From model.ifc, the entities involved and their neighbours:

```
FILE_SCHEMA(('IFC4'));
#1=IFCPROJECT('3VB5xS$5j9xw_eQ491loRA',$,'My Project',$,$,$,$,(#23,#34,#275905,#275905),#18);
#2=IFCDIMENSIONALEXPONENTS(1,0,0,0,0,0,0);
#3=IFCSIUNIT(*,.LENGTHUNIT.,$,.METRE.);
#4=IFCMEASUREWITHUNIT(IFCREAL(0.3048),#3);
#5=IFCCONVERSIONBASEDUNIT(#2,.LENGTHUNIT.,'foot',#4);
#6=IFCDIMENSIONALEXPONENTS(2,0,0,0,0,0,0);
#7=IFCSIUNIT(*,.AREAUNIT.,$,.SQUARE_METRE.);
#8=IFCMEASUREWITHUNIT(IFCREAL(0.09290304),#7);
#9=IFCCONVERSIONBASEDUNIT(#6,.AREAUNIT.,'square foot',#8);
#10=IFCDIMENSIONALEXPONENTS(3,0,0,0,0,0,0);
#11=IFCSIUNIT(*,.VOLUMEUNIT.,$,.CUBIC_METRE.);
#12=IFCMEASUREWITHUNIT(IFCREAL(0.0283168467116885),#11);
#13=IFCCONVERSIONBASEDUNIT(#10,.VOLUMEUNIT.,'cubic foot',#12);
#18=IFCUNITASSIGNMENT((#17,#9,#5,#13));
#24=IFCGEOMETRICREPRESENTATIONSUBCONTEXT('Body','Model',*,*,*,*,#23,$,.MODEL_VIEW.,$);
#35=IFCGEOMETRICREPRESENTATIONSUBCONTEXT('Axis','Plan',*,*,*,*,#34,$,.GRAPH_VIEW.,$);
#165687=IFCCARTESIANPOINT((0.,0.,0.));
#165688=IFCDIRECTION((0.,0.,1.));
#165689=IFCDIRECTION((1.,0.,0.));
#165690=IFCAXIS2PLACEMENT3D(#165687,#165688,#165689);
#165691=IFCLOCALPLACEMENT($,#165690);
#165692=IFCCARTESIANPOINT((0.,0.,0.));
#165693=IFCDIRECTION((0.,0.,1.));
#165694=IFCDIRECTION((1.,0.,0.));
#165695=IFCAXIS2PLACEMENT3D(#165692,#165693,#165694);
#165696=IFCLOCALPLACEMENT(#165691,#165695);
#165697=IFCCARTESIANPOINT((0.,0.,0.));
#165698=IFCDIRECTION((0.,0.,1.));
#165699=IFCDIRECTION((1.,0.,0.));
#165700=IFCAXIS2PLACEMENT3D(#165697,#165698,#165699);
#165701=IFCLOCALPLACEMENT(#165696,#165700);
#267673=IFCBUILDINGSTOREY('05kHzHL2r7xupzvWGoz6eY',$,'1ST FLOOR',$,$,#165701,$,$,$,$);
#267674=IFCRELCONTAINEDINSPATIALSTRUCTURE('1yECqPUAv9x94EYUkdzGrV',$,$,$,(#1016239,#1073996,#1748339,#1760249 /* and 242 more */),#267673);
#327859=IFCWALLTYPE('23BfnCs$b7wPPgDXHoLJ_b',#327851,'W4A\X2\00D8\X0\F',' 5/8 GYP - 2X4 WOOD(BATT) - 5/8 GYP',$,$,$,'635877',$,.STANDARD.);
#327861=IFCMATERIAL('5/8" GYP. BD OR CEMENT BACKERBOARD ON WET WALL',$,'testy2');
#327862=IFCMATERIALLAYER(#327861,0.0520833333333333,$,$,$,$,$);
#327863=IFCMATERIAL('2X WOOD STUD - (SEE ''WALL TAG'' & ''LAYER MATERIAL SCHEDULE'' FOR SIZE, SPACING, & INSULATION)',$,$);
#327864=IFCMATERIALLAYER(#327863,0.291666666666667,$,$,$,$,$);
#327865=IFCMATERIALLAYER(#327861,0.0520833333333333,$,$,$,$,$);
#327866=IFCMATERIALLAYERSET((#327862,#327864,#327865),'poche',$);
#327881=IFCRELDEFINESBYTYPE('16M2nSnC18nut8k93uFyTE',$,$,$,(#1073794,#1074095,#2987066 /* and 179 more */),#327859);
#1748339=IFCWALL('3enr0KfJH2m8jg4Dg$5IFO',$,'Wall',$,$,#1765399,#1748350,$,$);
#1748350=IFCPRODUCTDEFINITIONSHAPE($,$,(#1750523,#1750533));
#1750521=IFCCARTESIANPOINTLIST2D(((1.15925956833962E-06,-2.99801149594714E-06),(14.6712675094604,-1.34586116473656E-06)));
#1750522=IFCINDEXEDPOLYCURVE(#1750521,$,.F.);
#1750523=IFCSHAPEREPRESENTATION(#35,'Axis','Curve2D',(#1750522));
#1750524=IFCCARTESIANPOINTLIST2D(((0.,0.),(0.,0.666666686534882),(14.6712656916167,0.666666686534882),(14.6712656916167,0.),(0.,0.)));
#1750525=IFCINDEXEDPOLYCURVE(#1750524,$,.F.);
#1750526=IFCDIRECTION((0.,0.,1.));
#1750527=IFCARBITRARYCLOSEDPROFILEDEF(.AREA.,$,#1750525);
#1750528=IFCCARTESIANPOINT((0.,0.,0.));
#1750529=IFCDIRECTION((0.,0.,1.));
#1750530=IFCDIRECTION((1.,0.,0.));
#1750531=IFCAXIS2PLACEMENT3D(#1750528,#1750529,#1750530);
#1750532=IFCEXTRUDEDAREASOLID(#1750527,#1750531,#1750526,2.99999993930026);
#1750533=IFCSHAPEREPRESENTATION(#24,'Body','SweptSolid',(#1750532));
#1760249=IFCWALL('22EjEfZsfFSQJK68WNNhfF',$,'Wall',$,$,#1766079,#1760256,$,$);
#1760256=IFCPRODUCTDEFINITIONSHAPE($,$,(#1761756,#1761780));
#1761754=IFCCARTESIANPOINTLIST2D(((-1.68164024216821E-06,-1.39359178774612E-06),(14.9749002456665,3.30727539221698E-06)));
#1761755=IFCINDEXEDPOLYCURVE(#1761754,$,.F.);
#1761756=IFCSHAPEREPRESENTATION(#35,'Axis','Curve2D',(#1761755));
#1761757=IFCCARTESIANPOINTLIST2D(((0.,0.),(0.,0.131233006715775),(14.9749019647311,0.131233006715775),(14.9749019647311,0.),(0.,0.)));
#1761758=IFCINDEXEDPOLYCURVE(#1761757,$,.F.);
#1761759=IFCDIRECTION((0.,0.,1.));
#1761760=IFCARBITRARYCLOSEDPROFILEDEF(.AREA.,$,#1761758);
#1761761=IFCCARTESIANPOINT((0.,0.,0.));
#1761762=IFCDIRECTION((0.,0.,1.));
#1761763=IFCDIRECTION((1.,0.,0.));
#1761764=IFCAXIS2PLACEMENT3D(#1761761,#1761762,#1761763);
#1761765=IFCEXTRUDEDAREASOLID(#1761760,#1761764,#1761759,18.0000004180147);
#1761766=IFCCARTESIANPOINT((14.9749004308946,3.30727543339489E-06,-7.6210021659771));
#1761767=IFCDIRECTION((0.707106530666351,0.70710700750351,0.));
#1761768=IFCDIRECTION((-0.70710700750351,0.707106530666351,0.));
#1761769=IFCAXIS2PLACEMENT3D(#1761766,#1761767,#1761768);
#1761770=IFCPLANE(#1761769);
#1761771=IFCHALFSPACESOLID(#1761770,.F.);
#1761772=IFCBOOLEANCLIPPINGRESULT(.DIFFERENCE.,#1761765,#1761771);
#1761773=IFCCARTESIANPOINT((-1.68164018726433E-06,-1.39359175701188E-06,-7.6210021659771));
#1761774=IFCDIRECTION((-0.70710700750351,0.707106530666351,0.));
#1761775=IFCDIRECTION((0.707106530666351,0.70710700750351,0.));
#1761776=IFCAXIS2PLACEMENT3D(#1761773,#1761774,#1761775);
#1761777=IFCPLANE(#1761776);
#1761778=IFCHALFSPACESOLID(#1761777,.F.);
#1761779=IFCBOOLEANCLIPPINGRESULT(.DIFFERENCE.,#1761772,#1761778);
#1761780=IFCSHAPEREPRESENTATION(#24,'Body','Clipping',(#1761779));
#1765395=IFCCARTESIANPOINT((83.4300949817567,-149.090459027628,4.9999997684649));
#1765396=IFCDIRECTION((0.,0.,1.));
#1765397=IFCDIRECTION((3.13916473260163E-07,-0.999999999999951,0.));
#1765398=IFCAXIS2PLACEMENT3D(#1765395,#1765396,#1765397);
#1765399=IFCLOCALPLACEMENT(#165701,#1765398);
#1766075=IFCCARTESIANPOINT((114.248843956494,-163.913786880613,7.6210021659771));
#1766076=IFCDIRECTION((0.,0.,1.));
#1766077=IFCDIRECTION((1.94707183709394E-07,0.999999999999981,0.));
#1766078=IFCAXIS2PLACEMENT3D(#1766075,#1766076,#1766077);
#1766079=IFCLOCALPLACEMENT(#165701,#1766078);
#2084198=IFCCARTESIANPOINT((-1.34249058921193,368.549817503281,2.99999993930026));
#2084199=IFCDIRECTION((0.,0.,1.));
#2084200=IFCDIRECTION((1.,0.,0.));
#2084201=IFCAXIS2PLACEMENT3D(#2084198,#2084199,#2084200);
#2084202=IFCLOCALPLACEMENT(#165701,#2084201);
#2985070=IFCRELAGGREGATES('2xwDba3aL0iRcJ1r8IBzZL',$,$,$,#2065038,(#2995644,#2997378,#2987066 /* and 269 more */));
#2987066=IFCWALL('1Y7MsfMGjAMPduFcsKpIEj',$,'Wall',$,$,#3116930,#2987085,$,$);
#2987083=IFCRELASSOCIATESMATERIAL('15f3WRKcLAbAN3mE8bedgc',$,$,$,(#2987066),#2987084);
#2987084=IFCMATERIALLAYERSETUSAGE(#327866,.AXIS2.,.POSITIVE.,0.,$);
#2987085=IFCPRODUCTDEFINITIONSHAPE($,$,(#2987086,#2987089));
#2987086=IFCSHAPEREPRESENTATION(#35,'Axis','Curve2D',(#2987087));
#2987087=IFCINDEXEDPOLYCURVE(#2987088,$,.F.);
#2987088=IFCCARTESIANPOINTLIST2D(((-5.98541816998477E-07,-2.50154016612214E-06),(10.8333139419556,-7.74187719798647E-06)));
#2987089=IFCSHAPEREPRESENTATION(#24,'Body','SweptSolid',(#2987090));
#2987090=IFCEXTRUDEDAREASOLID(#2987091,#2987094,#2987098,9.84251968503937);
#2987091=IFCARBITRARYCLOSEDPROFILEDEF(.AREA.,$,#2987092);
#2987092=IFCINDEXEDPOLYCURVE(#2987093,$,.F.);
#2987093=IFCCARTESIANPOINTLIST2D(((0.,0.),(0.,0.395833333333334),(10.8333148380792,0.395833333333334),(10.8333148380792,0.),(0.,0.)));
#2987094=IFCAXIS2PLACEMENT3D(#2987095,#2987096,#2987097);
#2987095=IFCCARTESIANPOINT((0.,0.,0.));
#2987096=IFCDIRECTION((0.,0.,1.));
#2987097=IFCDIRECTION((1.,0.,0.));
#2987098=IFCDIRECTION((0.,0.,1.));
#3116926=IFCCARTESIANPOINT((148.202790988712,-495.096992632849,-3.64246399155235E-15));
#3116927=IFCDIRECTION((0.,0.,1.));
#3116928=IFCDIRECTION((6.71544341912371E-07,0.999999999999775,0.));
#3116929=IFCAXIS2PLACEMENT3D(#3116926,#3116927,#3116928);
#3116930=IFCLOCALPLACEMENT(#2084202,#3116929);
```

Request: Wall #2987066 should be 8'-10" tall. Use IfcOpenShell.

```python
import ifcopenshell
import ifcopenshell.geom
import ifcopenshell.util.representation
import ifcopenshell.util.shape
import ifcopenshell.util.unit

model = ifcopenshell.open("model.ifc")
unit_scale = ifcopenshell.util.unit.calculate_unit_scale(model)
settings = ifcopenshell.geom.settings()


def volume(element):
    """Net volume in cubic metres, openings subtracted."""
    shape = ifcopenshell.geom.create_shape(settings, element)
    return ifcopenshell.util.shape.get_volume(shape.geometry)


wall = model.by_id(2987066)
before = volume(wall)

body = ifcopenshell.util.representation.get_representation(wall, "Model", "Body")
solid = body.Items[0]
old_height = solid.Depth
solid.Depth = 106 * 0.0254 / unit_scale
after = volume(wall)

print(f"height {old_height:g} -> {solid.Depth:g}, volume {before:.3f} -> {after:.3f} m3")

model.write("model_updated.ifc")
```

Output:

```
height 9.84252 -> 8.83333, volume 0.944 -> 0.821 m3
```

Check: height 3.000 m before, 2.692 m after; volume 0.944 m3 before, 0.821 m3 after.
